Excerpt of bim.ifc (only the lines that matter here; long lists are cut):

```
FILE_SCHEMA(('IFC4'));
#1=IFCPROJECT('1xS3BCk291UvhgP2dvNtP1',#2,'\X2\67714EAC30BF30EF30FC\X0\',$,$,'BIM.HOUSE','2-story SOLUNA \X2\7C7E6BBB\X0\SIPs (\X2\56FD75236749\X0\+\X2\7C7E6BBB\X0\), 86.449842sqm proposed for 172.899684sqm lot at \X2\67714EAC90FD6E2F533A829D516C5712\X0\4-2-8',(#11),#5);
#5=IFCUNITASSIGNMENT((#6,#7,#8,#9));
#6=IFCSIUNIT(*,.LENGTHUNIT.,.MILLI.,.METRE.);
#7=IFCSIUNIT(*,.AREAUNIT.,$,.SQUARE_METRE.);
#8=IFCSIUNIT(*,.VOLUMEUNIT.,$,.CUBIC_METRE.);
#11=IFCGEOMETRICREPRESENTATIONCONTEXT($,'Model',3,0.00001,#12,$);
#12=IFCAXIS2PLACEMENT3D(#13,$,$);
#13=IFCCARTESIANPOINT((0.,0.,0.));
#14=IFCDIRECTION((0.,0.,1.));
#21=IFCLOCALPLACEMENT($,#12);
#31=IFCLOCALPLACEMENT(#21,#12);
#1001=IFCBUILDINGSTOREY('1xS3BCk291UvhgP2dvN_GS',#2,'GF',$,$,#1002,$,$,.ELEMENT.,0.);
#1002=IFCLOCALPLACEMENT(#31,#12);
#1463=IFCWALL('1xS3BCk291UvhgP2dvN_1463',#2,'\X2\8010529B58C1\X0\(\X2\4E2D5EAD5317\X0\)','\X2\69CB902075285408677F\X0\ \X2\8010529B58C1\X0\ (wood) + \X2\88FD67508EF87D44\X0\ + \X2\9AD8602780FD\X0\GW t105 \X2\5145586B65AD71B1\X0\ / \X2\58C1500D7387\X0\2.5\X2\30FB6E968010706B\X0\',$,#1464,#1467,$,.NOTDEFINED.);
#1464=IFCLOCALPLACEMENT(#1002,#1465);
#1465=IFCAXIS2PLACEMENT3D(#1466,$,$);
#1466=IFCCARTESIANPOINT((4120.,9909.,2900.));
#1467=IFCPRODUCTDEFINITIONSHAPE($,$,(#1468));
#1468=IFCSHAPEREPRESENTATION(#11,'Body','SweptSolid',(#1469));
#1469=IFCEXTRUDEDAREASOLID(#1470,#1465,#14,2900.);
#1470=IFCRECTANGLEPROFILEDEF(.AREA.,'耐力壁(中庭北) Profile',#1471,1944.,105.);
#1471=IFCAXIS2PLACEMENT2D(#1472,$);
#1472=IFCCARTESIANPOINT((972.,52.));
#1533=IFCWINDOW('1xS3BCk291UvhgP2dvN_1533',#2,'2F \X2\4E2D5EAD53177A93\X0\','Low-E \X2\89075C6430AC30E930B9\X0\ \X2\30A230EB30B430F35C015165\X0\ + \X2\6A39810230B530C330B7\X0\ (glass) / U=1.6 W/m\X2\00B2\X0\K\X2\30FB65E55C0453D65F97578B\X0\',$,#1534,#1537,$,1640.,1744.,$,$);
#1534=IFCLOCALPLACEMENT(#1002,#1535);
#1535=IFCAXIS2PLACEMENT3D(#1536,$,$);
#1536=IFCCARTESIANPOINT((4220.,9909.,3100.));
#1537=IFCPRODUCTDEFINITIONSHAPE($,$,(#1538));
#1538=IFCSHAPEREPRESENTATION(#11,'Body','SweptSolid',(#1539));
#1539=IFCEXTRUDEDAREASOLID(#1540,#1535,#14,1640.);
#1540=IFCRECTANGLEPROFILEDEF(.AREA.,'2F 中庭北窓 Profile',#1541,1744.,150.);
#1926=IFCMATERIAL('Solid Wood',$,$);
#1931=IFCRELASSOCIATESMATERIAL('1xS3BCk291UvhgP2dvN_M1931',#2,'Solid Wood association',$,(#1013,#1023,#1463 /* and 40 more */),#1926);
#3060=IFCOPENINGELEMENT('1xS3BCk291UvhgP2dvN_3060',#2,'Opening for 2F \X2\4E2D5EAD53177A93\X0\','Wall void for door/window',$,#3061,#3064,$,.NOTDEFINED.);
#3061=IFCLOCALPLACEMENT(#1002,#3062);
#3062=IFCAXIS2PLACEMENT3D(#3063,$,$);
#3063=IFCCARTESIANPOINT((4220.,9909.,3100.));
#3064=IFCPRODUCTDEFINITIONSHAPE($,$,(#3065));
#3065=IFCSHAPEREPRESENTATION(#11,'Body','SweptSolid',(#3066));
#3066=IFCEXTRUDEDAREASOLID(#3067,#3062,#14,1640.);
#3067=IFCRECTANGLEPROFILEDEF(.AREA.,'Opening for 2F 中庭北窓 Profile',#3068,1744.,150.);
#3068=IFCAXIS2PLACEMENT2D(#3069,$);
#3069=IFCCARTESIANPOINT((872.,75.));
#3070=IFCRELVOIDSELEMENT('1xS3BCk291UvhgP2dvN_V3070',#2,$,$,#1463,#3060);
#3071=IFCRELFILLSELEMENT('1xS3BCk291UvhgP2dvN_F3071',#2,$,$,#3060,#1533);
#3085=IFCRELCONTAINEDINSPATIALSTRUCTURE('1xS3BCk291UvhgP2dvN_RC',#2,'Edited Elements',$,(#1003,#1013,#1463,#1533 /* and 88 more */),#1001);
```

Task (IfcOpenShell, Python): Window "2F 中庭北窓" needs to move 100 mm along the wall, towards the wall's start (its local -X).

```python
import ifcopenshell
import ifcopenshell.api.geometry
import ifcopenshell.util.placement

model = ifcopenshell.open("bim.ifc")

window = model.by_id(1533)
opening = window.FillsVoids[0].RelatingOpeningElement
wall = opening.VoidsElements[0].RelatingBuildingElement

wall_matrix = ifcopenshell.util.placement.get_local_placement(wall.ObjectPlacement)
shift = wall_matrix[:3, 0] * -100.0
before = ifcopenshell.util.placement.get_local_placement(window.ObjectPlacement)[:3, 3].copy()

# The window is not placed relative to its opening, so move both.
for product in (opening, window):
    matrix = ifcopenshell.util.placement.get_local_placement(product.ObjectPlacement)
    matrix[:3, 3] += shift
    ifcopenshell.api.geometry.edit_object_placement(model, product=product, matrix=matrix, is_si=False)

after = ifcopenshell.util.placement.get_local_placement(window.ObjectPlacement)[:3, 3]
print("window moved by", (after - before).round(3) + 0.0)

model.write("bim_rev.ifc")
```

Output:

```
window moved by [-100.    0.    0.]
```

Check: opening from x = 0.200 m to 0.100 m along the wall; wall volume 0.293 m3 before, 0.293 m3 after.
